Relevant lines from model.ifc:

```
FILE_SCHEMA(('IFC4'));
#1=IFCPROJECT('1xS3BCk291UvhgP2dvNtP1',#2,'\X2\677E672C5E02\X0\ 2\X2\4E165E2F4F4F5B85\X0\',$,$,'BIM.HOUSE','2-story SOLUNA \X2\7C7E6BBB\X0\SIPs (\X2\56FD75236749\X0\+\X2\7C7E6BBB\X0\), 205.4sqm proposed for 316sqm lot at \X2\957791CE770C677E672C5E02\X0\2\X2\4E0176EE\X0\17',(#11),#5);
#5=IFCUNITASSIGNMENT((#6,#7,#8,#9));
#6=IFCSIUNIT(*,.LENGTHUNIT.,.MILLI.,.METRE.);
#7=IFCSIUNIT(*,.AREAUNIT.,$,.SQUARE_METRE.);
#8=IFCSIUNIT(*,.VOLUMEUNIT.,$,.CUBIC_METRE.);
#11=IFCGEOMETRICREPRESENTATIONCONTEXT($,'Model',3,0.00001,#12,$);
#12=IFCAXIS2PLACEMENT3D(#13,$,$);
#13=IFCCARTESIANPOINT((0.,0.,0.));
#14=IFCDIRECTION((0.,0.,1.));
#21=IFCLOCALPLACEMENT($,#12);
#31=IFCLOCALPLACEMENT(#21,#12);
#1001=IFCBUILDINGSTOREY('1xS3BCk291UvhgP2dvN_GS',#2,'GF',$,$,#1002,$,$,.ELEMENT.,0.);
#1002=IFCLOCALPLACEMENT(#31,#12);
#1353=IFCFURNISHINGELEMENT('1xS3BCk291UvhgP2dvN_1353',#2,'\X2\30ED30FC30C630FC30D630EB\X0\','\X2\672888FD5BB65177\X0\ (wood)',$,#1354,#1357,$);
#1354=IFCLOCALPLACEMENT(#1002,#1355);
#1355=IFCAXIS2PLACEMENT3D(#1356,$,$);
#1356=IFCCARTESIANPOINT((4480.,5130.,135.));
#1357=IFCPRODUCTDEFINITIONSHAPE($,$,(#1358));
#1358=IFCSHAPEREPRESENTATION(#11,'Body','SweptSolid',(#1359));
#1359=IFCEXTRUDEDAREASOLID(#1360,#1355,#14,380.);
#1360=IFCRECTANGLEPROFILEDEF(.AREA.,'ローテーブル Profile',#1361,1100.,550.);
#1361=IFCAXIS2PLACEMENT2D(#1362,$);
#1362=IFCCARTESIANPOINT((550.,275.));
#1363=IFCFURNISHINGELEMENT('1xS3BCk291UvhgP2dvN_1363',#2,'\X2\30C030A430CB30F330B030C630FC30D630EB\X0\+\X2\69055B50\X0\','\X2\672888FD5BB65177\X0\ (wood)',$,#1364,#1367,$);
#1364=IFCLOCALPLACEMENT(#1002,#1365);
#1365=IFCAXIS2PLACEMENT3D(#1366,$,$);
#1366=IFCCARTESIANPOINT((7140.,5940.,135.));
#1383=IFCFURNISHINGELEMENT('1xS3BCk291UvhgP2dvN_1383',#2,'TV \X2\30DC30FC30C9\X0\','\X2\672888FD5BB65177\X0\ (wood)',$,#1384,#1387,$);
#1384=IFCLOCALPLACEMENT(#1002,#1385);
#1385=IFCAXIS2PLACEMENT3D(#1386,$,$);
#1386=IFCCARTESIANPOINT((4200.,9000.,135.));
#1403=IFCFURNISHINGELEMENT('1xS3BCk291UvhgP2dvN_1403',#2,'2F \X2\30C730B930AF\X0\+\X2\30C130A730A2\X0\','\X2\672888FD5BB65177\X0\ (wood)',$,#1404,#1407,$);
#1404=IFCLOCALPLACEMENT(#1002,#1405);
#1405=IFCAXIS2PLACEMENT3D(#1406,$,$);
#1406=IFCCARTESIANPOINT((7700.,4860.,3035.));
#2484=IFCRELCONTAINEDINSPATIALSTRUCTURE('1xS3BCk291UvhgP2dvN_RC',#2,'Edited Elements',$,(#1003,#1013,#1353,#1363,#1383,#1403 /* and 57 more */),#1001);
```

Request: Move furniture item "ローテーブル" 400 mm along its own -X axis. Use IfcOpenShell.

```python
import ifcopenshell
import ifcopenshell.api.geometry
import ifcopenshell.util.placement

model = ifcopenshell.open("model.ifc")

item = model.by_id(1353)
matrix = ifcopenshell.util.placement.get_local_placement(item.ObjectPlacement)
matrix[:3, 3] -= matrix[:3, 0] * 400.0
ifcopenshell.api.geometry.edit_object_placement(model, product=item, matrix=matrix, is_si=False)

print(ifcopenshell.util.placement.get_local_placement(item.ObjectPlacement).round(3) + 0.0)

model.write("model_v2.ifc")
```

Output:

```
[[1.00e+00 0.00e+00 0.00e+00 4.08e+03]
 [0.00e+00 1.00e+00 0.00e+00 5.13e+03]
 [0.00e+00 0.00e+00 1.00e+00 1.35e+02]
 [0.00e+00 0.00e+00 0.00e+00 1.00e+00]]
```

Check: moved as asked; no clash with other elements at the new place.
